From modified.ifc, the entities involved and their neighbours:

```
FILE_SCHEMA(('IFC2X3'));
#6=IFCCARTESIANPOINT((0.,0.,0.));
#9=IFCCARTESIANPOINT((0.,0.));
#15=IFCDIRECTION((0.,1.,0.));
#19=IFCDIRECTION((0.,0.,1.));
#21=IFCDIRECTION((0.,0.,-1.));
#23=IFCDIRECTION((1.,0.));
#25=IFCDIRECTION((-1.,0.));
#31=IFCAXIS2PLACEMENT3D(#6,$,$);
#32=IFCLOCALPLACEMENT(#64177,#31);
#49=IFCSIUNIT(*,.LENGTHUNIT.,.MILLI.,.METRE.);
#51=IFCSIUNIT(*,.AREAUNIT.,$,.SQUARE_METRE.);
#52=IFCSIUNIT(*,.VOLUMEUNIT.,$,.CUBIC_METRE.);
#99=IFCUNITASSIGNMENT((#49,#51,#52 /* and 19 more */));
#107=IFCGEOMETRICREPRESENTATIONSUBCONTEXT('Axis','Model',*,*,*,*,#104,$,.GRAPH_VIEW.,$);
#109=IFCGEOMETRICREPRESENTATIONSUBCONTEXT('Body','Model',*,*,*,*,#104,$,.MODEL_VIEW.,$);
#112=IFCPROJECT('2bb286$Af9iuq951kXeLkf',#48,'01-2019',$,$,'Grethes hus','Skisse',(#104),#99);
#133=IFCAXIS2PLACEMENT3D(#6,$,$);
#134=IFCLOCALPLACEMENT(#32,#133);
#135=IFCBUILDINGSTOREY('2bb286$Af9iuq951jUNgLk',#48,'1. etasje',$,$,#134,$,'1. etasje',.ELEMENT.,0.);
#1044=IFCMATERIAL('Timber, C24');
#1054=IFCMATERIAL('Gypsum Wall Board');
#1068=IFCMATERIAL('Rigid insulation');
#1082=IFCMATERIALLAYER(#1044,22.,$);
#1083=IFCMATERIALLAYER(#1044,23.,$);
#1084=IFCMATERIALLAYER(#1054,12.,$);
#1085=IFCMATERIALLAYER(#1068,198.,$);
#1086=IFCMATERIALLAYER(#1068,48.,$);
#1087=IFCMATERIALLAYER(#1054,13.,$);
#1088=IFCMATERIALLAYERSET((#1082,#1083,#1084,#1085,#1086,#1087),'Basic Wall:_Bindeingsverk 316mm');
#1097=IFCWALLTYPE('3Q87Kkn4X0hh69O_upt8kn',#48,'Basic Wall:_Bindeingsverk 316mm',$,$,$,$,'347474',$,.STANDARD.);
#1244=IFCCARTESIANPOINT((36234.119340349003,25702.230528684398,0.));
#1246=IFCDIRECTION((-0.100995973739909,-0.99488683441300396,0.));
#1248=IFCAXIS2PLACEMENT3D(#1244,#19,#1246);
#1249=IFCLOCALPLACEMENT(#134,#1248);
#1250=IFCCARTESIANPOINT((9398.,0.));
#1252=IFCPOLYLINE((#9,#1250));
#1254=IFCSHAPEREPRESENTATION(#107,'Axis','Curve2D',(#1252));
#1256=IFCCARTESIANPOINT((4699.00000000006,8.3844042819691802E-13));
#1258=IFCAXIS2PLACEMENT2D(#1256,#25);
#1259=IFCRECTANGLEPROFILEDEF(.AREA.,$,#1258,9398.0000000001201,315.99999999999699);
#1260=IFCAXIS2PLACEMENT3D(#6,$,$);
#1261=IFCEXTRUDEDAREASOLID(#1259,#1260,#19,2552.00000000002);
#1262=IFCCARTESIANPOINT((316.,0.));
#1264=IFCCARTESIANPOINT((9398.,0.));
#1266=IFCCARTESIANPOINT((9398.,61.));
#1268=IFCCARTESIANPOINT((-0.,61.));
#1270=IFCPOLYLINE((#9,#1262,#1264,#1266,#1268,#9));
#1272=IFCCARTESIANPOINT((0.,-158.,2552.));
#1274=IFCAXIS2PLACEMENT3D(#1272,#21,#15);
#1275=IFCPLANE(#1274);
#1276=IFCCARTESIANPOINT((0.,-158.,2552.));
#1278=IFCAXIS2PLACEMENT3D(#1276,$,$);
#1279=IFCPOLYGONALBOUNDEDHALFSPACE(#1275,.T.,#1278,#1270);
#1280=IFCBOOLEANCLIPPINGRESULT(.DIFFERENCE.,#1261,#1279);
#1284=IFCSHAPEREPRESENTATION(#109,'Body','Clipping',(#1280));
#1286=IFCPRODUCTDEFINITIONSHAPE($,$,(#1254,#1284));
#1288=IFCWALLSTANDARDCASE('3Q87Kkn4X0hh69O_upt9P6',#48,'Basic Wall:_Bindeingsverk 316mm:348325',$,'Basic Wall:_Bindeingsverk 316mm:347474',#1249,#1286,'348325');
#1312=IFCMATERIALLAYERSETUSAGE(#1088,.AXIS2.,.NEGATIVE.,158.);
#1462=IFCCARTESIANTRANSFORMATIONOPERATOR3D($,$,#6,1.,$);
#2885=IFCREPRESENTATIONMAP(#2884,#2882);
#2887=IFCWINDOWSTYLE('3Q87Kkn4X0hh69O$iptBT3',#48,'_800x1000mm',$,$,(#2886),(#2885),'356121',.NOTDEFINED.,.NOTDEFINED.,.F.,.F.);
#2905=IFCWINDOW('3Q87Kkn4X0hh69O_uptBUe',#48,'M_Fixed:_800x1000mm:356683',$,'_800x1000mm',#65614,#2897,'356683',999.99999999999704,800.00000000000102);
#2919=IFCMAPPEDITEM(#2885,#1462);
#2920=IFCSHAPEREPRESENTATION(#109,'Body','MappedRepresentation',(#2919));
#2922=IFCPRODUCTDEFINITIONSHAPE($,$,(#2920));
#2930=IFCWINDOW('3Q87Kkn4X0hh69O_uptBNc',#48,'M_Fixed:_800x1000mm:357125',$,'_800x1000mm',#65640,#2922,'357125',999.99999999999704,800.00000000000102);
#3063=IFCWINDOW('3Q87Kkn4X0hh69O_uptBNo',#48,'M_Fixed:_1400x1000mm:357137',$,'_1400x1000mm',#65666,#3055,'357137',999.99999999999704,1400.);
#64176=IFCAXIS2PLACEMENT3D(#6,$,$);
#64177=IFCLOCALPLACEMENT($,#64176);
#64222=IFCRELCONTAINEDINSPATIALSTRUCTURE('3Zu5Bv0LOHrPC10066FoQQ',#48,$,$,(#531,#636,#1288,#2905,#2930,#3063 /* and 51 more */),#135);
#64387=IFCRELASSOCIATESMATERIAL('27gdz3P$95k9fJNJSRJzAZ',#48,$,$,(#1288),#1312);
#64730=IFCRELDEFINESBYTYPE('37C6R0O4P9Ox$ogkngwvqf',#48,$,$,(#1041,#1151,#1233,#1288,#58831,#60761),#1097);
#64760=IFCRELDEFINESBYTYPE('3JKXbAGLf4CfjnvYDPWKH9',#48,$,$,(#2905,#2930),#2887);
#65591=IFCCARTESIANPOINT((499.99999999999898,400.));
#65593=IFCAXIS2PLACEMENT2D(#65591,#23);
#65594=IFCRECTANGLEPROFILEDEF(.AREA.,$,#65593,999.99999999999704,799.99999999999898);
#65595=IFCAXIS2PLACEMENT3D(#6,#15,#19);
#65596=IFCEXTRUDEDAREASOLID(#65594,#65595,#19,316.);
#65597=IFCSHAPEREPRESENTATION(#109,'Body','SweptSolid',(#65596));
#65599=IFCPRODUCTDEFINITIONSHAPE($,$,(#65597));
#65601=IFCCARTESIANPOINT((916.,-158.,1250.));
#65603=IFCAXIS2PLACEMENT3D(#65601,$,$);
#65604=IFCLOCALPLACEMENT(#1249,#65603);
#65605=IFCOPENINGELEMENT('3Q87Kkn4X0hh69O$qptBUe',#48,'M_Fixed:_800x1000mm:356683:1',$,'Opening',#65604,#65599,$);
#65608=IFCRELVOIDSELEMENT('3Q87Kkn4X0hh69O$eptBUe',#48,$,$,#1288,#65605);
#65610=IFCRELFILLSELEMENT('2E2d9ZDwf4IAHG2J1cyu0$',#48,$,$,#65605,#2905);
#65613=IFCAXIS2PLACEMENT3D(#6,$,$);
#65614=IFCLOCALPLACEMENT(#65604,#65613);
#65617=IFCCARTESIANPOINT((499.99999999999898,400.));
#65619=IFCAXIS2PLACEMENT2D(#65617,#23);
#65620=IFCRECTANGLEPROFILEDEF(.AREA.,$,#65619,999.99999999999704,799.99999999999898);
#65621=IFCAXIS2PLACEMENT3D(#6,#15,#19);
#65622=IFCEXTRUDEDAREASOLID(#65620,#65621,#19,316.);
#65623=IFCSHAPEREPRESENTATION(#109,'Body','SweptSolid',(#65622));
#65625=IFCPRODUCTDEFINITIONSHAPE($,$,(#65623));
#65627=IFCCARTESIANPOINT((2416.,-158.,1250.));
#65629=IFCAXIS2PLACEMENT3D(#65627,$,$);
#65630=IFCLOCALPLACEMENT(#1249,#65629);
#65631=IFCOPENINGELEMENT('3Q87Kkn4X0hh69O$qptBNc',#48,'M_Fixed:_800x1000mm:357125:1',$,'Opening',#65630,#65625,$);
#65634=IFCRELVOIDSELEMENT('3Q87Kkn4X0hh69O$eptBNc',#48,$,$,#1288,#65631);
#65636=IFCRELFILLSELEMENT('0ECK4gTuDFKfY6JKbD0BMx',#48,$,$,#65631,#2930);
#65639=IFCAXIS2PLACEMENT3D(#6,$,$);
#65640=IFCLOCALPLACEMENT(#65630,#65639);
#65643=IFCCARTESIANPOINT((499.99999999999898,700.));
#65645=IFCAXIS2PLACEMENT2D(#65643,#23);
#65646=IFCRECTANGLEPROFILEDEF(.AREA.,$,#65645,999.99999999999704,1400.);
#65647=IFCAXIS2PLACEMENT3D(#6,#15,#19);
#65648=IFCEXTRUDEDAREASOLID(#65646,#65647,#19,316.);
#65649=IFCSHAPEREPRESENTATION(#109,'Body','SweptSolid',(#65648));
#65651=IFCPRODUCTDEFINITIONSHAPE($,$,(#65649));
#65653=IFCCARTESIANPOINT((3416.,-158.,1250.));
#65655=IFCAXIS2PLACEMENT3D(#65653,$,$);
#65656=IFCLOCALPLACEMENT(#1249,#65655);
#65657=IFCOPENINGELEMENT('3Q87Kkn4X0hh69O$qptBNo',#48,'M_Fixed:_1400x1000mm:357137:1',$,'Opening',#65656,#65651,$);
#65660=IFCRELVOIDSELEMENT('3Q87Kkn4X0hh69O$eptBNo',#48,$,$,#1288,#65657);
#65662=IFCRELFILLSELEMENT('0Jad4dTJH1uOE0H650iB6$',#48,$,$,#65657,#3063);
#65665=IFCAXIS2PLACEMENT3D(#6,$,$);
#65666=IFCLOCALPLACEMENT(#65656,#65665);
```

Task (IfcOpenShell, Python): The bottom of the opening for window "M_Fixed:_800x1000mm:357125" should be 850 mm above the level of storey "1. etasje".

```python
import numpy as np
import ifcopenshell
import ifcopenshell.api.geometry
import ifcopenshell.geom
import ifcopenshell.util.element
import ifcopenshell.util.placement
import ifcopenshell.util.shape
import ifcopenshell.util.unit

model = ifcopenshell.open("modified.ifc")
unit_scale = ifcopenshell.util.unit.calculate_unit_scale(model)

window = model.by_guid("3Q87Kkn4X0hh69O_uptBNc")
opening = window.FillsVoids[0].RelatingOpeningElement
storey = ifcopenshell.util.element.get_container(window, ifc_class="IfcBuildingStorey")
level = ifcopenshell.util.placement.get_local_placement(storey.ObjectPlacement)[2, 3]

# The opening's origin need not be at the sill, so measure its lowest point.
shape = ifcopenshell.geom.create_shape(ifcopenshell.geom.settings(), opening)
bottom = ifcopenshell.util.shape.get_shape_bottom_elevation(shape, shape.geometry) / unit_scale
dz = level + 0.85 / unit_scale - bottom

shift = np.array([0.0, 0.0, dz])
# The window is placed relative to its opening, so it follows when the opening moves.
matrix = ifcopenshell.util.placement.get_local_placement(opening.ObjectPlacement)
matrix[:3, 3] += shift
ifcopenshell.api.geometry.edit_object_placement(
    model, product=opening, matrix=matrix, is_si=False, should_transform_children=True
)

print(f"moved by {dz * unit_scale:+.3f} m")

model.write("modified_edited.ifc")
```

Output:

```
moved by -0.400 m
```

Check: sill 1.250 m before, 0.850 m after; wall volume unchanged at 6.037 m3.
